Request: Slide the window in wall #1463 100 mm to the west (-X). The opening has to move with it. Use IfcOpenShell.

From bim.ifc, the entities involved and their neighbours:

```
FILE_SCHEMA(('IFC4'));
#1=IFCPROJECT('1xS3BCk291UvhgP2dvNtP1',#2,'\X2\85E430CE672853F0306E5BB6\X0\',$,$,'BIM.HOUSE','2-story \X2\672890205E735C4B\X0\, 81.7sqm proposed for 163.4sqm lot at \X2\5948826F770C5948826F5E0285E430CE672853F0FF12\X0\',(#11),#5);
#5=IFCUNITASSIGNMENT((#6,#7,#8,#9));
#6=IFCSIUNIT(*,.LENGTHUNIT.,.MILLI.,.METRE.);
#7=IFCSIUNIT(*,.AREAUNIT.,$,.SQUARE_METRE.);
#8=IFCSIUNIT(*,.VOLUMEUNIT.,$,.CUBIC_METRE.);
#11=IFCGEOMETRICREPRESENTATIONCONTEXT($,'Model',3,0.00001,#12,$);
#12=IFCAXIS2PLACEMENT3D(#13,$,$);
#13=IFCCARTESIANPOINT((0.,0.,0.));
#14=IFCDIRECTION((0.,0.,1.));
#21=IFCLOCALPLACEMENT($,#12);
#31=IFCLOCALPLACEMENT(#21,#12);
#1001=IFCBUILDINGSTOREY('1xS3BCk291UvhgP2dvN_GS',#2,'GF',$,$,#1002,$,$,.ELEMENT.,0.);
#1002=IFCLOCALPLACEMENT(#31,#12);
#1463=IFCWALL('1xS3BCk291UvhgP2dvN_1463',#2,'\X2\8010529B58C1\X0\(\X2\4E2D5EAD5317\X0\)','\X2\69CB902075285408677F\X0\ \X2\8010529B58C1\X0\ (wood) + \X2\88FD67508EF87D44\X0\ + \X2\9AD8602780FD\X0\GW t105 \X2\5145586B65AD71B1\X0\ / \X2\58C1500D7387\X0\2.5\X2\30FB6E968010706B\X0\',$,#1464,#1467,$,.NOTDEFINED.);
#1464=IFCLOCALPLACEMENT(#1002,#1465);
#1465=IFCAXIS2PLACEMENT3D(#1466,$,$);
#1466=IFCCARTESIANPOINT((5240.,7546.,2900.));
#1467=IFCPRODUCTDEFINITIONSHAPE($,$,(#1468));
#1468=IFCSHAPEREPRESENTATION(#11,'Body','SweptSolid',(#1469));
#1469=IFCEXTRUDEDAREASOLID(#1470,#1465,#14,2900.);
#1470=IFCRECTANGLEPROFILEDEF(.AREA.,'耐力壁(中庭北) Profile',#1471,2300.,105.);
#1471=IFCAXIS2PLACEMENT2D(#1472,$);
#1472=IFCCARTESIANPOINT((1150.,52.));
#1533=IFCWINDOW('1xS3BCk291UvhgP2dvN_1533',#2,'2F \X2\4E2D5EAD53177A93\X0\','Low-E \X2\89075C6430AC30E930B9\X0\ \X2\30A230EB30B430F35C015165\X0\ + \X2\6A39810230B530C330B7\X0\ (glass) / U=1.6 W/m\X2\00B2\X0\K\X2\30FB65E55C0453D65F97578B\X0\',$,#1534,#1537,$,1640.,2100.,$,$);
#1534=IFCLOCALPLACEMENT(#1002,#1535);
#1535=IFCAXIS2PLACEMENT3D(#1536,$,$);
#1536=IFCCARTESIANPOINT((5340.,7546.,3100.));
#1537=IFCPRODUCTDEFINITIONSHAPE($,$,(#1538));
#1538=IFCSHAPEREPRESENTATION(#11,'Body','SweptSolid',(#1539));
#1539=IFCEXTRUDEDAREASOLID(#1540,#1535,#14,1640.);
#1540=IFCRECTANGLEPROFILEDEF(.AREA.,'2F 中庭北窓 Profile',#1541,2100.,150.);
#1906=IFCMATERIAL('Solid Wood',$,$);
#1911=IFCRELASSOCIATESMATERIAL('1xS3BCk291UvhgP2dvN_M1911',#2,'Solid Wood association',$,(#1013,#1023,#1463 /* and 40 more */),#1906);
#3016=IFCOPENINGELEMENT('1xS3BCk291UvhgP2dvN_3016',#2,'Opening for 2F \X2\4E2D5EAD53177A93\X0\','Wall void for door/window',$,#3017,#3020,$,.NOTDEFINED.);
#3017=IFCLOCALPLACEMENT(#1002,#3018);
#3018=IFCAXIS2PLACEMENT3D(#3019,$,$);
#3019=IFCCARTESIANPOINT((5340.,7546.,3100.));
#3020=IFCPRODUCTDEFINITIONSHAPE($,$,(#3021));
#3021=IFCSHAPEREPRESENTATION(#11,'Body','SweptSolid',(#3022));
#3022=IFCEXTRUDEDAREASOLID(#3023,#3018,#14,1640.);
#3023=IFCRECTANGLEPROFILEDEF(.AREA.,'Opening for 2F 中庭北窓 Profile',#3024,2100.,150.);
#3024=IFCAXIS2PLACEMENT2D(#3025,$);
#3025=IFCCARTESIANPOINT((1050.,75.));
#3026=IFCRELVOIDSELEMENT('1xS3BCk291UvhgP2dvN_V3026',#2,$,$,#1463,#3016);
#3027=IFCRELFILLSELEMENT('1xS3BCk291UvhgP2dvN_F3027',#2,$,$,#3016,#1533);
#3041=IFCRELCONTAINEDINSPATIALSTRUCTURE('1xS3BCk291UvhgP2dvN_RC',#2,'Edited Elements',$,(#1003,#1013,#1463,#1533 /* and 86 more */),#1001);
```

```python
import ifcopenshell
import ifcopenshell.api.geometry
import ifcopenshell.util.placement
import ifcopenshell.util.unit

model = ifcopenshell.open("bim.ifc")
unit_scale = ifcopenshell.util.unit.calculate_unit_scale(model)

window = model.by_id(1533)
opening = window.FillsVoids[0].RelatingOpeningElement
wall = opening.VoidsElements[0].RelatingBuildingElement

wall_matrix = ifcopenshell.util.placement.get_local_placement(wall.ObjectPlacement)
shift = wall_matrix[:3, 0] * -0.1 / unit_scale
before = ifcopenshell.util.placement.get_local_placement(window.ObjectPlacement)[:3, 3].copy()

# The window is not placed relative to its opening, so move both.
for product in (opening, window):
    matrix = ifcopenshell.util.placement.get_local_placement(product.ObjectPlacement)
    matrix[:3, 3] += shift
    ifcopenshell.api.geometry.edit_object_placement(model, product=product, matrix=matrix, is_si=False)

after = ifcopenshell.util.placement.get_local_placement(window.ObjectPlacement)[:3, 3]
print("window moved by", (after - before).round(3) + 0.0)

model.write("bim_updated.ifc")
```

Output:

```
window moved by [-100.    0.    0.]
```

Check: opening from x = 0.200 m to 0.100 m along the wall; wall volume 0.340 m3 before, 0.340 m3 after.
